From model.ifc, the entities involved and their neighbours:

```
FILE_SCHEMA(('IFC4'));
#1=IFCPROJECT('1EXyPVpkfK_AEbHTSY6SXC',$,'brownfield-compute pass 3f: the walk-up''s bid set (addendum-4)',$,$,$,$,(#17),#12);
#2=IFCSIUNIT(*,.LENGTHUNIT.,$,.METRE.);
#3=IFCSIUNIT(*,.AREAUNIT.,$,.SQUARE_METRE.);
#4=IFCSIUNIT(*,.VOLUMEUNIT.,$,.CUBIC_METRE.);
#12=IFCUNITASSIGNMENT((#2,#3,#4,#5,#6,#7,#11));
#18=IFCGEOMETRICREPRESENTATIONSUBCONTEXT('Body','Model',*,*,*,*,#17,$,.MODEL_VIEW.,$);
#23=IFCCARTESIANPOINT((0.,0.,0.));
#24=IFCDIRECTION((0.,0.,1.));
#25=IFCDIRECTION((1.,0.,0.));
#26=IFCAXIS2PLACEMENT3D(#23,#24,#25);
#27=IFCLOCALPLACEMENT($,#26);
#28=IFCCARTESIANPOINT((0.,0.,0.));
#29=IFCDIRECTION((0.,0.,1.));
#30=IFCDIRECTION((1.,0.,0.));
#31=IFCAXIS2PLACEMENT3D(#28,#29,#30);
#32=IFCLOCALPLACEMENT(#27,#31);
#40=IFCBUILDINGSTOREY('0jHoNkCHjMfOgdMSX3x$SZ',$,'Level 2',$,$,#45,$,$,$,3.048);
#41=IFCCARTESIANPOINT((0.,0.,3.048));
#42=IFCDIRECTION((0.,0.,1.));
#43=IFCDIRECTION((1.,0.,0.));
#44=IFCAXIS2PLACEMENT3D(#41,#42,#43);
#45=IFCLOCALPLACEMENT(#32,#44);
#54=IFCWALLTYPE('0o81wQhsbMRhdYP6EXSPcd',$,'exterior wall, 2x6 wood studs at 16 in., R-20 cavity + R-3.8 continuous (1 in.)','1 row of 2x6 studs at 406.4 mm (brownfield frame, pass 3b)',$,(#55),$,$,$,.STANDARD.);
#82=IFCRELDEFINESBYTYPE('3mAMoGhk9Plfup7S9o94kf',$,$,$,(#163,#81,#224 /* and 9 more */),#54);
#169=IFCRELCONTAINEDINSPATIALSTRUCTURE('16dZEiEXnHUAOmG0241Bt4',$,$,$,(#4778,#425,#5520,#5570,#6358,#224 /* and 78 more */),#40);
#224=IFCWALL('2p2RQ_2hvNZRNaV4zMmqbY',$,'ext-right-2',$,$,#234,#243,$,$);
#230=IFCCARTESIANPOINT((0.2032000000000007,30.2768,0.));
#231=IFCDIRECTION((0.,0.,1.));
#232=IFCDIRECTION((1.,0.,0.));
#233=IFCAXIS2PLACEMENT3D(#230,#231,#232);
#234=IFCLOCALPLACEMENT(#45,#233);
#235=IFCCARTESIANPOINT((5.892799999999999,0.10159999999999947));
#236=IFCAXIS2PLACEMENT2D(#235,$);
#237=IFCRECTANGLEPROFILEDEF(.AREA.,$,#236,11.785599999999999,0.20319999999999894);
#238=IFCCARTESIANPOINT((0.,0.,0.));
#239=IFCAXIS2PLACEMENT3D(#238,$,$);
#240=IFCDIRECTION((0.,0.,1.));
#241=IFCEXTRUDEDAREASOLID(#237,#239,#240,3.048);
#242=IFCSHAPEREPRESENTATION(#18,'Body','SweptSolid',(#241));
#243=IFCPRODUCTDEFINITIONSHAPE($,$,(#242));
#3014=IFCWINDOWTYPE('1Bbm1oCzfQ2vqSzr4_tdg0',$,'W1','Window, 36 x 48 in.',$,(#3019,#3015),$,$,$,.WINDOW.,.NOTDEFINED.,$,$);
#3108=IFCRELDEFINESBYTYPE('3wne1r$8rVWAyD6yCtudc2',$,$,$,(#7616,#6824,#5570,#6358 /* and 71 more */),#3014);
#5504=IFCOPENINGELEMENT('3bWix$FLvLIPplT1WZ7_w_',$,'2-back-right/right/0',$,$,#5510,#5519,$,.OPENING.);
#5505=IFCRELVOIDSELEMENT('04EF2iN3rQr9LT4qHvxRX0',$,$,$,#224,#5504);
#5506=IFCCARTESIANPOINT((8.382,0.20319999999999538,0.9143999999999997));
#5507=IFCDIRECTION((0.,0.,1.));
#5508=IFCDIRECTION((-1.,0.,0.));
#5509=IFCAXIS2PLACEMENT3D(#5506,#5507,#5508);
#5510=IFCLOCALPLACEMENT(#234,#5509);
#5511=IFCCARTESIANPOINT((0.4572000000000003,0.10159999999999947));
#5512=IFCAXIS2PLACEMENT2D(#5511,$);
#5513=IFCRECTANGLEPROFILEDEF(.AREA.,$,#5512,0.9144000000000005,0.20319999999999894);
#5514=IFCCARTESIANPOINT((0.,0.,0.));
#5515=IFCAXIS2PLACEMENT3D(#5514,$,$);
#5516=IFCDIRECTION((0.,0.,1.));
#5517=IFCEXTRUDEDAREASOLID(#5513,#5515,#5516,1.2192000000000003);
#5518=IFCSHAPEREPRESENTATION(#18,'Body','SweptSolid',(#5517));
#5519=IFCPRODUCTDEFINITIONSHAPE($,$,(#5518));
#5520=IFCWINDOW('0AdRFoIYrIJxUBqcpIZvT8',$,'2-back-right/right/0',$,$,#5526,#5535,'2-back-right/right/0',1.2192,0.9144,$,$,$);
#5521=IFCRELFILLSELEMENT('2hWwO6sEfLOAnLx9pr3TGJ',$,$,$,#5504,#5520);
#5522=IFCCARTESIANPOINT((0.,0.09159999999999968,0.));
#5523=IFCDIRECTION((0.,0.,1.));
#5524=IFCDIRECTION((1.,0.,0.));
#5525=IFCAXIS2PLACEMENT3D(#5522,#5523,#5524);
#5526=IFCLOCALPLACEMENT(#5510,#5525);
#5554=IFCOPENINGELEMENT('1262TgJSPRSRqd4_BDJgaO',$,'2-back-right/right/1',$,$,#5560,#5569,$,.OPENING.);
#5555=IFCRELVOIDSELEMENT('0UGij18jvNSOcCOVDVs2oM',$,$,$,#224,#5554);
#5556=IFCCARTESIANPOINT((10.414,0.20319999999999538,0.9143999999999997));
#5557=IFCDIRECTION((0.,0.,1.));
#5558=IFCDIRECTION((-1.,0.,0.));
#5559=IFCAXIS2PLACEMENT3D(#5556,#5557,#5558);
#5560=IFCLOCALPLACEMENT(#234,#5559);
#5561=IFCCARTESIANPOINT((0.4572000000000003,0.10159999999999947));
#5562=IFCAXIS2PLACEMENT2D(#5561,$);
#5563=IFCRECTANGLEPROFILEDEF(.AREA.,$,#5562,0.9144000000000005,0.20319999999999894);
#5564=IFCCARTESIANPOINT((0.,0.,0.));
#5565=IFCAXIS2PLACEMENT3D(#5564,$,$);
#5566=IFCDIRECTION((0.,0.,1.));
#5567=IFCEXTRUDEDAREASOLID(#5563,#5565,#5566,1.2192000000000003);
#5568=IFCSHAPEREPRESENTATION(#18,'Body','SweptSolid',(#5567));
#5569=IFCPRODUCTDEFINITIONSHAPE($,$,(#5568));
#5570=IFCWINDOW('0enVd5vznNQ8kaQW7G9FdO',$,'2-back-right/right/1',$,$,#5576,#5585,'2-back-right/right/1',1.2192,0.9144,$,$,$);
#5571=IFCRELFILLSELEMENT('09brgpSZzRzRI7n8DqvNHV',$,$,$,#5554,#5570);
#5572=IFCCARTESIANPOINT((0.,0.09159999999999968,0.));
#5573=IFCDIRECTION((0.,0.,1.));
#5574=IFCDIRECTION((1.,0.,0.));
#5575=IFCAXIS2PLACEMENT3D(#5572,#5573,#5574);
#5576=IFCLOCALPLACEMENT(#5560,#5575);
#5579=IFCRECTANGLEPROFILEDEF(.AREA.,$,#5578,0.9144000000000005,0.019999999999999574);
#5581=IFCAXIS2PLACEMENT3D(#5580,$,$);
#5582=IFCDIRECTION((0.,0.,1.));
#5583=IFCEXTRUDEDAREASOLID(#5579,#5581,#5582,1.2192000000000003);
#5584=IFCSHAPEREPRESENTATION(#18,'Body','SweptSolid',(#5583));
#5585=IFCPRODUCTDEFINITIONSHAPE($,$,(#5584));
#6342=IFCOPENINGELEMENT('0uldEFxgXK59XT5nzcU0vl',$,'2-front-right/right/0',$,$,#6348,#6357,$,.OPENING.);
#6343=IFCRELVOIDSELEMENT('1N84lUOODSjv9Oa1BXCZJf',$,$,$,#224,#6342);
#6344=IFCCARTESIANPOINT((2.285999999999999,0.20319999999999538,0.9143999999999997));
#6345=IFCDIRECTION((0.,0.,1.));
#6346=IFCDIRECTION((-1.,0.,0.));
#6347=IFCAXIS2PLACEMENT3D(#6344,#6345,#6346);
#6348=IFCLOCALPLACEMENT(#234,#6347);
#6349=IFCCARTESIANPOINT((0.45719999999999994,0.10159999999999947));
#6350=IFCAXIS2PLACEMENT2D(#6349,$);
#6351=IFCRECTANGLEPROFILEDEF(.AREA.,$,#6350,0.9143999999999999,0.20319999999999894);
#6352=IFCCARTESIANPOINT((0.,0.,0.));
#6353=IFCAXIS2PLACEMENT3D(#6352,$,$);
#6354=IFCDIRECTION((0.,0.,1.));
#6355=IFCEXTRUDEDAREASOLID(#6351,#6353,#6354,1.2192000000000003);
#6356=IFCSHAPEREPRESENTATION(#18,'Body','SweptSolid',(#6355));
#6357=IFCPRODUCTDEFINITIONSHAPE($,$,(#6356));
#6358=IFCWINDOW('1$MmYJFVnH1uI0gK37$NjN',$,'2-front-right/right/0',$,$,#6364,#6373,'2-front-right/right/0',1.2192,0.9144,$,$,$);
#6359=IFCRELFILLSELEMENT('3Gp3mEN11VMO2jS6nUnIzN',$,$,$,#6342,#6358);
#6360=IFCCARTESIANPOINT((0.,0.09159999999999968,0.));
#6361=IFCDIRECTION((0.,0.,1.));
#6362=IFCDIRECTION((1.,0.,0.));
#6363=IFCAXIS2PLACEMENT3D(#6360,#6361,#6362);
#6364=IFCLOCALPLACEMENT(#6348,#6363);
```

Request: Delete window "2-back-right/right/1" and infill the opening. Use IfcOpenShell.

```python
import ifcopenshell
import ifcopenshell.api.feature
import ifcopenshell.api.root
import ifcopenshell.geom
import ifcopenshell.util.shape

model = ifcopenshell.open("model.ifc")
settings = ifcopenshell.geom.settings()


def volume(element):
    """Net volume in cubic metres, openings subtracted."""
    shape = ifcopenshell.geom.create_shape(settings, element)
    return ifcopenshell.util.shape.get_volume(shape.geometry)


window = model.by_guid("0enVd5vznNQ8kaQW7G9FdO")
opening = window.FillsVoids[0].RelatingOpeningElement
wall = opening.VoidsElements[0].RelatingBuildingElement
before = volume(wall)

ifcopenshell.api.root.remove_product(model, product=window)
ifcopenshell.api.feature.remove_feature(model, feature=opening)

after = volume(wall)

print(f"wall volume {before:.3f} -> {after:.3f} m3")

model.write("model_rev.ifc")
```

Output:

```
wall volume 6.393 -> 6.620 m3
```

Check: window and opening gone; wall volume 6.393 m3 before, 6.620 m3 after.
